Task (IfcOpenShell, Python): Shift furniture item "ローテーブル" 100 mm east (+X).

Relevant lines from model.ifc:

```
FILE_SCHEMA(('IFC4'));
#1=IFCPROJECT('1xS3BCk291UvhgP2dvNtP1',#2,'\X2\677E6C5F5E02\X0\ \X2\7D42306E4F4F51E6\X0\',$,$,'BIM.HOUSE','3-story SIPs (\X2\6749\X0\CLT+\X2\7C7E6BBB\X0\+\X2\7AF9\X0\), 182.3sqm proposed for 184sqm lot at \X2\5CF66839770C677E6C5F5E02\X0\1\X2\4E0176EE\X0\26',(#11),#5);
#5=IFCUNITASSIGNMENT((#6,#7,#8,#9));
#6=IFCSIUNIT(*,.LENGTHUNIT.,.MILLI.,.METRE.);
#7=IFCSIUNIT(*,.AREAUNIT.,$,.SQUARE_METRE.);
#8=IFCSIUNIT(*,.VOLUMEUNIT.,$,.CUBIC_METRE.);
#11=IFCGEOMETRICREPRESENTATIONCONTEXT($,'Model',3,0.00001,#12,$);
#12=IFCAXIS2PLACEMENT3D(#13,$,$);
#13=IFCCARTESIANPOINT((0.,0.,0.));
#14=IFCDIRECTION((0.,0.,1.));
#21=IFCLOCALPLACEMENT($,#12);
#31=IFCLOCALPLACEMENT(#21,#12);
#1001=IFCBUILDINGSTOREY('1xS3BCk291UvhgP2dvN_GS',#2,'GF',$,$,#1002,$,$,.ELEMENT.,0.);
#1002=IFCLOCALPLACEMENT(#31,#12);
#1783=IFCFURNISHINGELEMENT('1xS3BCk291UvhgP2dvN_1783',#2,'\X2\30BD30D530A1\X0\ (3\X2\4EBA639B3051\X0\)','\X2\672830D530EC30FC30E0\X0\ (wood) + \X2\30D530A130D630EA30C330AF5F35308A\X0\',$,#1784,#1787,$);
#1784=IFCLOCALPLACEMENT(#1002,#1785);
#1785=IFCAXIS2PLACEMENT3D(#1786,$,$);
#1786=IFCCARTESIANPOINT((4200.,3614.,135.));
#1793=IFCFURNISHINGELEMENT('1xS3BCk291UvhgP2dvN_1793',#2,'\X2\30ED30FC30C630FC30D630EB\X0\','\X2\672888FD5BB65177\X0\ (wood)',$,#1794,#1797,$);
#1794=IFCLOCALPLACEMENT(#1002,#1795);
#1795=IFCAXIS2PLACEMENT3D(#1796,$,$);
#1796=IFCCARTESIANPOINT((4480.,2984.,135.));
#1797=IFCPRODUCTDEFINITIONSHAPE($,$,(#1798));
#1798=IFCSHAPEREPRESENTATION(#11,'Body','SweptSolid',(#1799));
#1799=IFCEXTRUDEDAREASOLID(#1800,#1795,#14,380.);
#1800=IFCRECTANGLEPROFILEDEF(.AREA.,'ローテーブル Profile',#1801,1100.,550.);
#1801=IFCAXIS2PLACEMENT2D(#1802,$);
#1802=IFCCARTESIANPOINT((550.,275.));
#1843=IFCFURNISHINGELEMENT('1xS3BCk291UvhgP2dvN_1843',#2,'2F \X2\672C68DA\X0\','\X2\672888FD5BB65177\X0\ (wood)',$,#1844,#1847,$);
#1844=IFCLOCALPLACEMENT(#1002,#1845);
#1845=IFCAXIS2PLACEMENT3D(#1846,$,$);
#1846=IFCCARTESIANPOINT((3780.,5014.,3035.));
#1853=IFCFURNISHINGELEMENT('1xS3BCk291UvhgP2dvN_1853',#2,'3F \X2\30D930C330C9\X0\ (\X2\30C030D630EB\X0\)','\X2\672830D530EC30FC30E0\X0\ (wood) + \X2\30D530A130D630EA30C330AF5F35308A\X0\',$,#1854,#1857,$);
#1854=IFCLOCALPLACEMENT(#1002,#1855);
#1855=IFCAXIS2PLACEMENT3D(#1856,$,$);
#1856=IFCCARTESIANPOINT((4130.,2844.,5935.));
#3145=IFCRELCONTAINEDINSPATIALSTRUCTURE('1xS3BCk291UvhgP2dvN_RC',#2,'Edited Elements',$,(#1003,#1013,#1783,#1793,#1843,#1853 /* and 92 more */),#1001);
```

```python
import ifcopenshell
import ifcopenshell.api.geometry
import ifcopenshell.util.placement
import ifcopenshell.util.unit

model = ifcopenshell.open("model.ifc")
unit_scale = ifcopenshell.util.unit.calculate_unit_scale(model)

item = model.by_guid("1xS3BCk291UvhgP2dvN_1793")
matrix = ifcopenshell.util.placement.get_local_placement(item.ObjectPlacement)
matrix[0, 3] += 0.1 / unit_scale
ifcopenshell.api.geometry.edit_object_placement(model, product=item, matrix=matrix, is_si=False)

print(ifcopenshell.util.placement.get_local_placement(item.ObjectPlacement).round(3) + 0.0)

model.write("model-out.ifc")
```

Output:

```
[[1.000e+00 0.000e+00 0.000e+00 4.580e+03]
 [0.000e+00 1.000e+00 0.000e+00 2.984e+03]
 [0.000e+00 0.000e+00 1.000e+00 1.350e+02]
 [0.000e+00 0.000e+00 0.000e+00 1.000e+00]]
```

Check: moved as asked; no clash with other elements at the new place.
